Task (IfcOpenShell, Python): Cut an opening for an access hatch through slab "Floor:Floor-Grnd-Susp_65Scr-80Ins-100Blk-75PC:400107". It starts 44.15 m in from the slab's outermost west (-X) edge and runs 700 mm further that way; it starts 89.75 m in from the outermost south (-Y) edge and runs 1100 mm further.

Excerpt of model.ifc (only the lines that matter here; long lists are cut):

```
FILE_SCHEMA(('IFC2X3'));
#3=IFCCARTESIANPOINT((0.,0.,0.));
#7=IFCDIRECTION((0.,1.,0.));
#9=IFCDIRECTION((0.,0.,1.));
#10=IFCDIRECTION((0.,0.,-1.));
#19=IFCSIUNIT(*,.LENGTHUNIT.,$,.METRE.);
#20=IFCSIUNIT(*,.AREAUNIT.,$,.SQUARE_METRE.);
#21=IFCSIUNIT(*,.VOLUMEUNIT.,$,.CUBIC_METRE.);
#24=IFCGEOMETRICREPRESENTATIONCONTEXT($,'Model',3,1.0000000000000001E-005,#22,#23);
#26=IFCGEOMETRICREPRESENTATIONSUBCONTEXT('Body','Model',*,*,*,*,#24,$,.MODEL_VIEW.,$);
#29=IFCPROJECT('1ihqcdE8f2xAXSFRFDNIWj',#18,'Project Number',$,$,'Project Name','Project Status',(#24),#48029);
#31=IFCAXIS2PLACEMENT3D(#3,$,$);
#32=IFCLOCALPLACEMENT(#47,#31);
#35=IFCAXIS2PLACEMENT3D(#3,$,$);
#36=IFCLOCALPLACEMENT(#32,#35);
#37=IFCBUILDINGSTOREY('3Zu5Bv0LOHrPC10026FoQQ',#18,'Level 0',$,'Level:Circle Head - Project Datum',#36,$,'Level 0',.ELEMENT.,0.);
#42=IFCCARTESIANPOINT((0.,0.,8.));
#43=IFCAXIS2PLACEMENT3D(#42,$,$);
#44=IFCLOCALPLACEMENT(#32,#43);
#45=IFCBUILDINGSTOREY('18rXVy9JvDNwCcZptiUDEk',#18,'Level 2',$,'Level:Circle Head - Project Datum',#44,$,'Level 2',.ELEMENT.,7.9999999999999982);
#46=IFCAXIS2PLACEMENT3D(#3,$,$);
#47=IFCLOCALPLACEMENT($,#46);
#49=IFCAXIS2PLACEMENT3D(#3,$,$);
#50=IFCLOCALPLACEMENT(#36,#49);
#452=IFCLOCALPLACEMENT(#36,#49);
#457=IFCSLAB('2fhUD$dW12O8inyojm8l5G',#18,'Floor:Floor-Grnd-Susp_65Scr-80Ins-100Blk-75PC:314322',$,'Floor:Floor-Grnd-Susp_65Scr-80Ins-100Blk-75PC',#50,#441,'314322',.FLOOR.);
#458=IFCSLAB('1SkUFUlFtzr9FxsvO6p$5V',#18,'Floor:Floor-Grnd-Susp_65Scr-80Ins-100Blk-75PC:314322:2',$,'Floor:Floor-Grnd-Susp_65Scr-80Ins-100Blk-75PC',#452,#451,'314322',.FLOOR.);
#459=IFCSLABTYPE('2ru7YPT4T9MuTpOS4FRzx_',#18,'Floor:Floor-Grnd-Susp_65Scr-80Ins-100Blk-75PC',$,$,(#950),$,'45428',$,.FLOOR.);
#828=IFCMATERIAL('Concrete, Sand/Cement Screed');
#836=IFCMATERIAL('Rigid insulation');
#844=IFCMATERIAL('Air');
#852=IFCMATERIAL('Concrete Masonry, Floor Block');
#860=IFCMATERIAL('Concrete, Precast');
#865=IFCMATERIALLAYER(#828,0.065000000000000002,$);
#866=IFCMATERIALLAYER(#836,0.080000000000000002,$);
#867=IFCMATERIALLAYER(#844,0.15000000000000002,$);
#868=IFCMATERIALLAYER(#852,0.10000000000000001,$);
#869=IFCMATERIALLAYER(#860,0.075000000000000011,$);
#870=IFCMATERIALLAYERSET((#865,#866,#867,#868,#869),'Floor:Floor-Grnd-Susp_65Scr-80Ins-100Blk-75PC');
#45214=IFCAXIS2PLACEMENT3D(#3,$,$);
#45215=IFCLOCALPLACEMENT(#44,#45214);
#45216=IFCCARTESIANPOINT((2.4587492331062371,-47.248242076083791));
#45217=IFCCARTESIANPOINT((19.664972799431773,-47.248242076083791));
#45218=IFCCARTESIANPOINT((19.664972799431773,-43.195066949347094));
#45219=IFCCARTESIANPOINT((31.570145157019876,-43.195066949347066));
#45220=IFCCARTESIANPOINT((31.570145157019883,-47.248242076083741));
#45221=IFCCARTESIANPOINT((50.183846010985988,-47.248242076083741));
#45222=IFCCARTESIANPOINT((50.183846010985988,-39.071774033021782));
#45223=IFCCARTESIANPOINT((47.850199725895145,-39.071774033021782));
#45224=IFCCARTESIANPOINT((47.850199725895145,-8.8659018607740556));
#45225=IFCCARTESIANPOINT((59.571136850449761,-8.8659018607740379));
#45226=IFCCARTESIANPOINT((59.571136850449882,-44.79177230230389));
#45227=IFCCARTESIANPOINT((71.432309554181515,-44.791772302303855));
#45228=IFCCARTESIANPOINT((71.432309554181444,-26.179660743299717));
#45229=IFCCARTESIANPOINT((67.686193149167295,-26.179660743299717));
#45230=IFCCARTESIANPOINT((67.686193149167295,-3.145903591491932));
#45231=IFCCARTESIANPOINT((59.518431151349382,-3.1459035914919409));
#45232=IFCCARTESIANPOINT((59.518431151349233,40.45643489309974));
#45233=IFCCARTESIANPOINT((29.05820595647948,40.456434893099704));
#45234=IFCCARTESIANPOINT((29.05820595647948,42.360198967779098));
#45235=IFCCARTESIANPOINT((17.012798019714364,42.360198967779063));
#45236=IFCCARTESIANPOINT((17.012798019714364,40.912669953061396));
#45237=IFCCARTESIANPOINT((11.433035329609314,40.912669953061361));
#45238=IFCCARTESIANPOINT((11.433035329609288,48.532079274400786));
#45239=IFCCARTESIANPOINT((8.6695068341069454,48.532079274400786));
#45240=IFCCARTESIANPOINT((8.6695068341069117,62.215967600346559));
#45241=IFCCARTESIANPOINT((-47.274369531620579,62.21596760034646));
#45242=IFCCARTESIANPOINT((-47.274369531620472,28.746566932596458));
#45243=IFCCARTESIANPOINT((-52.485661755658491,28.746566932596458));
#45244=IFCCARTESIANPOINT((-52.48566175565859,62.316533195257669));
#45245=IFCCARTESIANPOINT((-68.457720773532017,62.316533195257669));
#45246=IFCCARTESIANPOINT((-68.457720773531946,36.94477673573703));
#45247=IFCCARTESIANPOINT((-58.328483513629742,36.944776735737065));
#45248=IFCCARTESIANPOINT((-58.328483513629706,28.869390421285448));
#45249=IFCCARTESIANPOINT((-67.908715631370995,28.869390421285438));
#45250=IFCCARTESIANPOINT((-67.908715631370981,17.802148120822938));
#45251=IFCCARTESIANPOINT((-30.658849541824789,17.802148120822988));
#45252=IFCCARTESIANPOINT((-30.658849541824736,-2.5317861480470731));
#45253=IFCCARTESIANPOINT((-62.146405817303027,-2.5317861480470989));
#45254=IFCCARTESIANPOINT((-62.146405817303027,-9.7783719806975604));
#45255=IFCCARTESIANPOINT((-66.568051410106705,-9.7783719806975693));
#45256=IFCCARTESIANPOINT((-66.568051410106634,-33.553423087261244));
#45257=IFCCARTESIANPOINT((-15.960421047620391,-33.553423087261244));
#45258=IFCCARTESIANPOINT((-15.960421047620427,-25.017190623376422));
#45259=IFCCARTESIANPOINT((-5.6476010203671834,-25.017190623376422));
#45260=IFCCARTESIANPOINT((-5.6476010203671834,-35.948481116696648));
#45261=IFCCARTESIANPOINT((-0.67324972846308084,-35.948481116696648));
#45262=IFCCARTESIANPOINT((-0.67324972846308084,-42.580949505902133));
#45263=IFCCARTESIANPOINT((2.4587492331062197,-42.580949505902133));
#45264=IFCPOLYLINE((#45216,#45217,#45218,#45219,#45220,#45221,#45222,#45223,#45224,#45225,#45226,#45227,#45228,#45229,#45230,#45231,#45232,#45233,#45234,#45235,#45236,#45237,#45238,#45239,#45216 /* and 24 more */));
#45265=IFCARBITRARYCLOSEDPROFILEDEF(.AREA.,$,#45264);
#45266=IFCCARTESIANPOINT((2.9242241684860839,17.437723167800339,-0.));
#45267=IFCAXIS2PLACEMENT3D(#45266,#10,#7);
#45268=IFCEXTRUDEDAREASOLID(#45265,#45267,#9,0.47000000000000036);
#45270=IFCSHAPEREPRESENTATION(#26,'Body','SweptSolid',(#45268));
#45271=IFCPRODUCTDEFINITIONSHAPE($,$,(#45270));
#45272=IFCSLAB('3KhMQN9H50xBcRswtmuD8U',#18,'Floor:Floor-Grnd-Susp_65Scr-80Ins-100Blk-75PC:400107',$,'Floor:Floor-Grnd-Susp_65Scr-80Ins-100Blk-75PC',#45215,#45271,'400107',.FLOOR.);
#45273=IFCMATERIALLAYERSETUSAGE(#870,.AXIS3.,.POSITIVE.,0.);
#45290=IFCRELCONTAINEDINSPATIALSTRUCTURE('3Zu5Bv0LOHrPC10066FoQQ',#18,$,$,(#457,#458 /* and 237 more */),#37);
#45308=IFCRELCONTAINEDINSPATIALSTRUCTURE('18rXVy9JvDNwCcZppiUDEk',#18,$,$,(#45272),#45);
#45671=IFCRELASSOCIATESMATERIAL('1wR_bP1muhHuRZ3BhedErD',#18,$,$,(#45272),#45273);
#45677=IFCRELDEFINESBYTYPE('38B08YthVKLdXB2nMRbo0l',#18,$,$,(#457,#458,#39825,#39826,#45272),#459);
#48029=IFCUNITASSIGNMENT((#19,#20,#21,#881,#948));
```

```python
import numpy as np
import ifcopenshell
import ifcopenshell.api.feature
import ifcopenshell.api.geometry
import ifcopenshell.api.root
import ifcopenshell.geom
import ifcopenshell.util.placement
import ifcopenshell.util.representation
import ifcopenshell.util.shape
import ifcopenshell.util.unit

model = ifcopenshell.open("model.ifc")
unit_scale = ifcopenshell.util.unit.calculate_unit_scale(model)
settings = ifcopenshell.geom.settings()


def volume(element):
    """Net volume in cubic metres, openings subtracted."""
    shape = ifcopenshell.geom.create_shape(settings, element)
    return ifcopenshell.util.shape.get_volume(shape.geometry)


slab = model.by_guid("3KhMQN9H50xBcRswtmuD8U")
before = volume(slab)

# Extent in the slab's own axes, in metres. The edges named are its -X and -Y sides.
slab_shape = ifcopenshell.geom.create_shape(settings, slab)
vertices = ifcopenshell.util.shape.get_vertices(slab_shape.geometry)
x_min, y_min, bottom = vertices.min(axis=0)
top = vertices[:, 2].max()

opening = ifcopenshell.api.root.create_entity(model, ifc_class="IfcOpeningElement", name="Access hatch opening")
context = ifcopenshell.util.representation.get_context(model, "Model", "Body", "MODEL_VIEW")
width, depth = 0.7, 1.1
outline = [(0.0, 0.0), (width, 0.0), (width, depth), (0.0, depth), (0.0, 0.0)]
# Overshoot both faces by 50 mm so the cut is clean.
shape = ifcopenshell.api.geometry.add_slab_representation(
    model, context=context, depth=top - bottom + 0.1, polyline=outline
)
ifcopenshell.api.geometry.assign_representation(model, product=opening, representation=shape)

matrix = ifcopenshell.util.placement.get_local_placement(slab.ObjectPlacement)
matrix[:, 3] = matrix @ np.append(np.array([x_min + 44.15, y_min + 89.75, bottom - 0.05]) / unit_scale, 1.0)
ifcopenshell.api.geometry.edit_object_placement(model, product=opening, matrix=matrix, is_si=False)
ifcopenshell.api.feature.add_feature(model, feature=opening, element=slab)

after = volume(slab)

print(f"slab volume {before:.3f} -> {after:.3f} m3")

model.write("model_rev.ifc")
```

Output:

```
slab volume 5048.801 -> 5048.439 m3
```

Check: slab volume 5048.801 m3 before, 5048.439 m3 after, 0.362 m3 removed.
